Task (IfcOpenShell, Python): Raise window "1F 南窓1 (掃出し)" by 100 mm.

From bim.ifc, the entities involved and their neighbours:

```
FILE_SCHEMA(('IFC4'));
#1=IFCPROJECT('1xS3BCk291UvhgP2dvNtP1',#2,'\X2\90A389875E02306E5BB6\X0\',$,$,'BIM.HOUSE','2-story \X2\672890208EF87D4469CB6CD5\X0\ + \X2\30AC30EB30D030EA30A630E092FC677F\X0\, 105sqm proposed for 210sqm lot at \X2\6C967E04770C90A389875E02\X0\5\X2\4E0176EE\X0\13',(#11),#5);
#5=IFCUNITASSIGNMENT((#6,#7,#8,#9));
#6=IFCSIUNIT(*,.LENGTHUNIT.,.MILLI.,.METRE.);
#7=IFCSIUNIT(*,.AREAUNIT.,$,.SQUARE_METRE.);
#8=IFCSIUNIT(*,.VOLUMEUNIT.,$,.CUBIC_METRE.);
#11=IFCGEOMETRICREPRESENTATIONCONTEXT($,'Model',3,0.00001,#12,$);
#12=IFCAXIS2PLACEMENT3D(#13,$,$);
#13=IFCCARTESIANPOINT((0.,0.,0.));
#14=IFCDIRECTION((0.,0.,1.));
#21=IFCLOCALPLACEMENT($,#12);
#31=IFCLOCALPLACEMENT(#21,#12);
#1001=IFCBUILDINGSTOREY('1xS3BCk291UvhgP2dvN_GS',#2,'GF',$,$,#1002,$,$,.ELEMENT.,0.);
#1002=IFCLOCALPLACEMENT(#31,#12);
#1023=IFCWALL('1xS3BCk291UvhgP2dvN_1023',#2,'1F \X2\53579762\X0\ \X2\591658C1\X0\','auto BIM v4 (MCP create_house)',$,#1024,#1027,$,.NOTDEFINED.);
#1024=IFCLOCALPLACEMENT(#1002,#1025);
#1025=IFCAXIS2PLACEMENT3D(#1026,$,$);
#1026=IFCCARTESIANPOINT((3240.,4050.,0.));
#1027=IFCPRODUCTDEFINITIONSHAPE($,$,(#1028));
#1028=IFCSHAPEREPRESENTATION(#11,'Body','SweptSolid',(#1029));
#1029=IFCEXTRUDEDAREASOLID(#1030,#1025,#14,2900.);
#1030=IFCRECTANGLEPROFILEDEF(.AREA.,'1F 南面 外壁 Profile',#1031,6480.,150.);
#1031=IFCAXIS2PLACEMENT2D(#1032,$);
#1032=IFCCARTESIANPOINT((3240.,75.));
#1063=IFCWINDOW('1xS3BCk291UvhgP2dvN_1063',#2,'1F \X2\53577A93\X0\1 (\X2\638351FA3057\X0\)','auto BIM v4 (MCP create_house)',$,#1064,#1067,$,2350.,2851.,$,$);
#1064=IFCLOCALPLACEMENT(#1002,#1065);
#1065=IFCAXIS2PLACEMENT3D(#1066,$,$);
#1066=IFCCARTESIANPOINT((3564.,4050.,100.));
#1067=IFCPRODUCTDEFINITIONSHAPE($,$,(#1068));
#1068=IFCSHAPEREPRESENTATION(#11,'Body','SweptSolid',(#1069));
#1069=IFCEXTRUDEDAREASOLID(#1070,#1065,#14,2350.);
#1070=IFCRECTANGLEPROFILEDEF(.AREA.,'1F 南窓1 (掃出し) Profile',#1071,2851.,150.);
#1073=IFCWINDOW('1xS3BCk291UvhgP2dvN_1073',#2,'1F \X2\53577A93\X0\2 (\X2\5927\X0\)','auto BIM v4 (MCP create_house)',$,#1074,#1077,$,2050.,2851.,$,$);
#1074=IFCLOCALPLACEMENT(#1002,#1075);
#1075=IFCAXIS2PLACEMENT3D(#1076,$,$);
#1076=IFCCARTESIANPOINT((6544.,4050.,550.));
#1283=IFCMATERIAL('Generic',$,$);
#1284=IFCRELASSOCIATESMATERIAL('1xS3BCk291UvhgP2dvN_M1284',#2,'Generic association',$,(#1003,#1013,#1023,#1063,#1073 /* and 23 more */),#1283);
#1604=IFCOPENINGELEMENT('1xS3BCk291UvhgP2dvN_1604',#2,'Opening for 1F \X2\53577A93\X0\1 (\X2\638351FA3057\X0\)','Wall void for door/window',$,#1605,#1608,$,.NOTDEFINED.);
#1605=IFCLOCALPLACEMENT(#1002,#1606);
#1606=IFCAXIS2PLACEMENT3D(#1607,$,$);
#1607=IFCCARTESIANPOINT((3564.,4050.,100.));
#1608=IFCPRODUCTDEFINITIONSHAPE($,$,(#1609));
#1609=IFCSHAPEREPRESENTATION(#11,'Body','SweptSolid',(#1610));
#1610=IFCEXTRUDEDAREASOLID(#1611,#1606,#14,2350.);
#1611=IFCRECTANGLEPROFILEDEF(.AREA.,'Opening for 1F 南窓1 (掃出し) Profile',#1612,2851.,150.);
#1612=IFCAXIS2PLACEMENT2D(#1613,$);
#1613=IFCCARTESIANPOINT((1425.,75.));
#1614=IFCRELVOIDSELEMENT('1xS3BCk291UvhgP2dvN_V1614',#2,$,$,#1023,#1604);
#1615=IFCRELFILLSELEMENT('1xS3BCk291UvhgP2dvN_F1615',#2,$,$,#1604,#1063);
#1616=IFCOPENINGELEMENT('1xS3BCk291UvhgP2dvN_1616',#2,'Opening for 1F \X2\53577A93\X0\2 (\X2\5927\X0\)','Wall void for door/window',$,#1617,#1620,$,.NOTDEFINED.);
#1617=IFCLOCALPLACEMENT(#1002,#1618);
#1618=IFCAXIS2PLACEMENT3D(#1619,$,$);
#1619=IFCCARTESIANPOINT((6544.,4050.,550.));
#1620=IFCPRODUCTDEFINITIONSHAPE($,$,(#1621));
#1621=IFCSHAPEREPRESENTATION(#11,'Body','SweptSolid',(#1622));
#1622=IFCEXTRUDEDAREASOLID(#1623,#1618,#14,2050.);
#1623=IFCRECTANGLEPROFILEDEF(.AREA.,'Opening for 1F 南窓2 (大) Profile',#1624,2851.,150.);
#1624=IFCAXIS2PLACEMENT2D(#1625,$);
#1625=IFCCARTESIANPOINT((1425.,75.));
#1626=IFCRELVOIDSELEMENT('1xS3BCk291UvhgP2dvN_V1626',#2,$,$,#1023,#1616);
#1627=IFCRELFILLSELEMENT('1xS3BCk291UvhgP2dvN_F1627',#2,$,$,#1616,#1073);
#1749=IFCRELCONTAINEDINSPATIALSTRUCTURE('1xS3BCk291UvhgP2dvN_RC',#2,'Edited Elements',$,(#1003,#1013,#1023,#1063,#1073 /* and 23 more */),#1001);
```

```python
import numpy as np
import ifcopenshell
import ifcopenshell.api.geometry
import ifcopenshell.util.placement
import ifcopenshell.util.unit

model = ifcopenshell.open("bim.ifc")
unit_scale = ifcopenshell.util.unit.calculate_unit_scale(model)

window = model.by_guid("1xS3BCk291UvhgP2dvN_1063")
opening = window.FillsVoids[0].RelatingOpeningElement
dz = 0.1 / unit_scale

shift = np.array([0.0, 0.0, dz])
# The window is not placed relative to its opening, so move both.
for product in (opening, window):
    matrix = ifcopenshell.util.placement.get_local_placement(product.ObjectPlacement)
    matrix[:3, 3] += shift
    ifcopenshell.api.geometry.edit_object_placement(model, product=product, matrix=matrix, is_si=False)

print(f"moved by {dz * unit_scale:+.3f} m")

model.write("bim-out.ifc")
```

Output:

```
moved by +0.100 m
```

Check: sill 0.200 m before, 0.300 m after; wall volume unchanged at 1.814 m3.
